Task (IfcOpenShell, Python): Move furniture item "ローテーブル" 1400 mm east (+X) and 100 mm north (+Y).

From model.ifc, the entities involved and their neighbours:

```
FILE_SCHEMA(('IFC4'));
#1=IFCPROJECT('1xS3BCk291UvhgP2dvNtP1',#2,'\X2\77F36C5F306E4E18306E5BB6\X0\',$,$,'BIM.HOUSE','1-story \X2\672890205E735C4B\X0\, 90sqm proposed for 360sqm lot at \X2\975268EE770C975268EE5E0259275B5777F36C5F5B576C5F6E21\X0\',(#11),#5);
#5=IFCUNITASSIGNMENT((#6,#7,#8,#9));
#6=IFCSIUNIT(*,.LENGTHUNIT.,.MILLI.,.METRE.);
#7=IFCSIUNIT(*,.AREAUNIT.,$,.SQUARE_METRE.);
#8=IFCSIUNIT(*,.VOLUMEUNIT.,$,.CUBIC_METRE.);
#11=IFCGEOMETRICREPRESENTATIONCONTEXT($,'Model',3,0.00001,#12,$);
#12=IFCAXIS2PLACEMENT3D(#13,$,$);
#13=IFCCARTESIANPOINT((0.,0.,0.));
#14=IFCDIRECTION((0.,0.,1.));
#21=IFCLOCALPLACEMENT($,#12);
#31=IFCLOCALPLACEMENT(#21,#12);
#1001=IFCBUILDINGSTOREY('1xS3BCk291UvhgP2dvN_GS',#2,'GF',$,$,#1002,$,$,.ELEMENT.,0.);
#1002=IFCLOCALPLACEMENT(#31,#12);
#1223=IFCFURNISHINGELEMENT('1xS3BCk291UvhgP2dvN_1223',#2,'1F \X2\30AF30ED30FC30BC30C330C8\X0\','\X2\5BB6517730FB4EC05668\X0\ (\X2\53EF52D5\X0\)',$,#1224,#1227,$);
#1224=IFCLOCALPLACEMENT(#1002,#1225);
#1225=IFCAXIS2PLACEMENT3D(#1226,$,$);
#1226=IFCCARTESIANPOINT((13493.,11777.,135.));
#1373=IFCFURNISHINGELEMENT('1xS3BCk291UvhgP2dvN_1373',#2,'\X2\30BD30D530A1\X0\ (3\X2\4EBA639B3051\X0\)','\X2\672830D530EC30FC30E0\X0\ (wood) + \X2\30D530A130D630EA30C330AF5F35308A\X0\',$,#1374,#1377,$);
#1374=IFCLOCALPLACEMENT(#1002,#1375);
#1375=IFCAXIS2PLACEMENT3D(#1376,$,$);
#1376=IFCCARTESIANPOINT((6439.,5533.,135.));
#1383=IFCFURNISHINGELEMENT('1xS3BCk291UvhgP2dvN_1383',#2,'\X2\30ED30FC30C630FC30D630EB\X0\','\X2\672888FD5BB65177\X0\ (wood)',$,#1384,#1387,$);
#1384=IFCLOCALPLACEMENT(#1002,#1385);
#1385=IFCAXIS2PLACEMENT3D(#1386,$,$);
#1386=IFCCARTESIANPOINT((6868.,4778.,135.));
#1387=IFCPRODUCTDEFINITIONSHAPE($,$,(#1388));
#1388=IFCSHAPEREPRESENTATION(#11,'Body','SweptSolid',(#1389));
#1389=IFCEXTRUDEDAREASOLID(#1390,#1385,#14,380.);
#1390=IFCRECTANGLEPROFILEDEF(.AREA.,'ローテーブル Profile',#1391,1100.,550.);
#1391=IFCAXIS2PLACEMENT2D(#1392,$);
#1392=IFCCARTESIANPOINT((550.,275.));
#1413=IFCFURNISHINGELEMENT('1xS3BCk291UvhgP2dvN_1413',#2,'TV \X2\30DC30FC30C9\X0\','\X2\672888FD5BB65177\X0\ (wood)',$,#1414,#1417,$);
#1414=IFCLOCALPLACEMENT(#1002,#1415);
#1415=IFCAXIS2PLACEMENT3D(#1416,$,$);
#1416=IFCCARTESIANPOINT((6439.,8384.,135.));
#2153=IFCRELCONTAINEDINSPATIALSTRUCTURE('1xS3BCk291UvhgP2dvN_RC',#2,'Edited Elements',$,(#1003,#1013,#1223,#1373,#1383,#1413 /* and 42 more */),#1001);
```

```python
import ifcopenshell
import ifcopenshell.api.geometry
import ifcopenshell.util.placement
import ifcopenshell.util.unit

model = ifcopenshell.open("model.ifc")
unit_scale = ifcopenshell.util.unit.calculate_unit_scale(model)

item = model.by_id(1383)
matrix = ifcopenshell.util.placement.get_local_placement(item.ObjectPlacement)
matrix[0, 3] += 1.4 / unit_scale
matrix[1, 3] += 0.1 / unit_scale
ifcopenshell.api.geometry.edit_object_placement(model, product=item, matrix=matrix, is_si=False)

print(ifcopenshell.util.placement.get_local_placement(item.ObjectPlacement).round(3) + 0.0)

model.write("model_rev.ifc")
```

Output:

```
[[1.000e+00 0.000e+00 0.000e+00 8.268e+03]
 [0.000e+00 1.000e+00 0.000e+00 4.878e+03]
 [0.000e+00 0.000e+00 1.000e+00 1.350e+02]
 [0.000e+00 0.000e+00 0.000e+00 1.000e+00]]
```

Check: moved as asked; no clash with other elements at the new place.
